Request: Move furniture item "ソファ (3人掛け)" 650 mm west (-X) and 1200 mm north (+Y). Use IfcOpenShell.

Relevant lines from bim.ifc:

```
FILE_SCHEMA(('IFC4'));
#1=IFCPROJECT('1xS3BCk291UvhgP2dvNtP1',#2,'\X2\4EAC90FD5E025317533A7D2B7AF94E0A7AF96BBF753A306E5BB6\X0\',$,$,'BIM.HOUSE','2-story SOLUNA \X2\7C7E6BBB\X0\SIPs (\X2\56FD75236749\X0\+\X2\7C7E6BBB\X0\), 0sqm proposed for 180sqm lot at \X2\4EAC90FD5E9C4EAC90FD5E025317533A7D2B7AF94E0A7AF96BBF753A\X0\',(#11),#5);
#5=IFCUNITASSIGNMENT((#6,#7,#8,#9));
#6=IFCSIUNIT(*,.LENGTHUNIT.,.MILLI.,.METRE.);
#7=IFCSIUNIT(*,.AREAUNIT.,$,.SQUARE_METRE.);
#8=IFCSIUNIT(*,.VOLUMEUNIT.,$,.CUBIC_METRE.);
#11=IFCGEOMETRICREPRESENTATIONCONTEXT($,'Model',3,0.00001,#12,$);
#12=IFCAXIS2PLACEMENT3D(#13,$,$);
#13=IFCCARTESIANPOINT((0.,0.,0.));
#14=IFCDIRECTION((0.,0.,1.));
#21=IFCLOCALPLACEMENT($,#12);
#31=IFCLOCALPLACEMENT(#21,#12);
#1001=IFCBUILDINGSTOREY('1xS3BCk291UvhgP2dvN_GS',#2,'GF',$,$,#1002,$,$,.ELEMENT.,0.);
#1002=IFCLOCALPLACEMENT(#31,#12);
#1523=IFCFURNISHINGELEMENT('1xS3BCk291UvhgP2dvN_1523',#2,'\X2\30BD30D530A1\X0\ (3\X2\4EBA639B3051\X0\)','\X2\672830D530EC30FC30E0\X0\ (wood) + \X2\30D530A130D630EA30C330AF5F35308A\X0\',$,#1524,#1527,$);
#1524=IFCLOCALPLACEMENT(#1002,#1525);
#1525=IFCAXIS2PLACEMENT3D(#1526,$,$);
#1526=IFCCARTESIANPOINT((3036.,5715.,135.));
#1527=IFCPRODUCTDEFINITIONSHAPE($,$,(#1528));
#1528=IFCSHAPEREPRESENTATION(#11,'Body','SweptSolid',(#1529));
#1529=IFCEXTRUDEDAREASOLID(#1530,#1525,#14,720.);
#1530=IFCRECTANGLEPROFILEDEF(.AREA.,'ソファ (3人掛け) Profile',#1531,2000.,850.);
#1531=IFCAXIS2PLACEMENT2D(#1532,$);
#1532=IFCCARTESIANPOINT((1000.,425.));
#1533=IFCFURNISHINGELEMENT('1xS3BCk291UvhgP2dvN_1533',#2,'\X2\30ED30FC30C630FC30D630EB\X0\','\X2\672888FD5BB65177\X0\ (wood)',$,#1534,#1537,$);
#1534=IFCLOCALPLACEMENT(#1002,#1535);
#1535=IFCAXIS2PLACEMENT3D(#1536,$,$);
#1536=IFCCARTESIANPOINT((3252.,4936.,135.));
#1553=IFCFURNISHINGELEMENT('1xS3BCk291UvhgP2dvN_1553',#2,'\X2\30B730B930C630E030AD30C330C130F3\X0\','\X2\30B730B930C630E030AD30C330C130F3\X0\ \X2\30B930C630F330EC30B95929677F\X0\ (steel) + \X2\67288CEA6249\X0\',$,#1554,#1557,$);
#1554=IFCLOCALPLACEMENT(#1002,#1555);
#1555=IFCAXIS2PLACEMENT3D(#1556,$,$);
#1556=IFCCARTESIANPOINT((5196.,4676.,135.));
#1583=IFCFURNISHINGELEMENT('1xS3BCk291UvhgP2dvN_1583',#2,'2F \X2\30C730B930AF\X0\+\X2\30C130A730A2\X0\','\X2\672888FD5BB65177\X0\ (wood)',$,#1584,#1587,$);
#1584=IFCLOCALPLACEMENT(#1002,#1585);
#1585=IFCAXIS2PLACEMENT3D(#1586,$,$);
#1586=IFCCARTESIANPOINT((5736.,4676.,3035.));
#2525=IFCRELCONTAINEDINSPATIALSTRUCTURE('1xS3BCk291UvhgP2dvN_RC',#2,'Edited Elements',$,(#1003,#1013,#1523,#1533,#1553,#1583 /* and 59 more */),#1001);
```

```python
import ifcopenshell
import ifcopenshell.api.geometry
import ifcopenshell.util.placement
import ifcopenshell.util.unit

model = ifcopenshell.open("bim.ifc")
unit_scale = ifcopenshell.util.unit.calculate_unit_scale(model)

item = model.by_guid("1xS3BCk291UvhgP2dvN_1523")
matrix = ifcopenshell.util.placement.get_local_placement(item.ObjectPlacement)
matrix[0, 3] -= 0.65 / unit_scale
matrix[1, 3] += 1.2 / unit_scale
ifcopenshell.api.geometry.edit_object_placement(model, product=item, matrix=matrix, is_si=False)

print(ifcopenshell.util.placement.get_local_placement(item.ObjectPlacement).round(3) + 0.0)

model.write("bim-out.ifc")
```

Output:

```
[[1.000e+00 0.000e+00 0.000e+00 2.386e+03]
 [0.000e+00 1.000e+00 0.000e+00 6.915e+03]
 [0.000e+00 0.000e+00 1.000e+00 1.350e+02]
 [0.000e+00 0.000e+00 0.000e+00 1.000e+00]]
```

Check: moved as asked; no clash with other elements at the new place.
